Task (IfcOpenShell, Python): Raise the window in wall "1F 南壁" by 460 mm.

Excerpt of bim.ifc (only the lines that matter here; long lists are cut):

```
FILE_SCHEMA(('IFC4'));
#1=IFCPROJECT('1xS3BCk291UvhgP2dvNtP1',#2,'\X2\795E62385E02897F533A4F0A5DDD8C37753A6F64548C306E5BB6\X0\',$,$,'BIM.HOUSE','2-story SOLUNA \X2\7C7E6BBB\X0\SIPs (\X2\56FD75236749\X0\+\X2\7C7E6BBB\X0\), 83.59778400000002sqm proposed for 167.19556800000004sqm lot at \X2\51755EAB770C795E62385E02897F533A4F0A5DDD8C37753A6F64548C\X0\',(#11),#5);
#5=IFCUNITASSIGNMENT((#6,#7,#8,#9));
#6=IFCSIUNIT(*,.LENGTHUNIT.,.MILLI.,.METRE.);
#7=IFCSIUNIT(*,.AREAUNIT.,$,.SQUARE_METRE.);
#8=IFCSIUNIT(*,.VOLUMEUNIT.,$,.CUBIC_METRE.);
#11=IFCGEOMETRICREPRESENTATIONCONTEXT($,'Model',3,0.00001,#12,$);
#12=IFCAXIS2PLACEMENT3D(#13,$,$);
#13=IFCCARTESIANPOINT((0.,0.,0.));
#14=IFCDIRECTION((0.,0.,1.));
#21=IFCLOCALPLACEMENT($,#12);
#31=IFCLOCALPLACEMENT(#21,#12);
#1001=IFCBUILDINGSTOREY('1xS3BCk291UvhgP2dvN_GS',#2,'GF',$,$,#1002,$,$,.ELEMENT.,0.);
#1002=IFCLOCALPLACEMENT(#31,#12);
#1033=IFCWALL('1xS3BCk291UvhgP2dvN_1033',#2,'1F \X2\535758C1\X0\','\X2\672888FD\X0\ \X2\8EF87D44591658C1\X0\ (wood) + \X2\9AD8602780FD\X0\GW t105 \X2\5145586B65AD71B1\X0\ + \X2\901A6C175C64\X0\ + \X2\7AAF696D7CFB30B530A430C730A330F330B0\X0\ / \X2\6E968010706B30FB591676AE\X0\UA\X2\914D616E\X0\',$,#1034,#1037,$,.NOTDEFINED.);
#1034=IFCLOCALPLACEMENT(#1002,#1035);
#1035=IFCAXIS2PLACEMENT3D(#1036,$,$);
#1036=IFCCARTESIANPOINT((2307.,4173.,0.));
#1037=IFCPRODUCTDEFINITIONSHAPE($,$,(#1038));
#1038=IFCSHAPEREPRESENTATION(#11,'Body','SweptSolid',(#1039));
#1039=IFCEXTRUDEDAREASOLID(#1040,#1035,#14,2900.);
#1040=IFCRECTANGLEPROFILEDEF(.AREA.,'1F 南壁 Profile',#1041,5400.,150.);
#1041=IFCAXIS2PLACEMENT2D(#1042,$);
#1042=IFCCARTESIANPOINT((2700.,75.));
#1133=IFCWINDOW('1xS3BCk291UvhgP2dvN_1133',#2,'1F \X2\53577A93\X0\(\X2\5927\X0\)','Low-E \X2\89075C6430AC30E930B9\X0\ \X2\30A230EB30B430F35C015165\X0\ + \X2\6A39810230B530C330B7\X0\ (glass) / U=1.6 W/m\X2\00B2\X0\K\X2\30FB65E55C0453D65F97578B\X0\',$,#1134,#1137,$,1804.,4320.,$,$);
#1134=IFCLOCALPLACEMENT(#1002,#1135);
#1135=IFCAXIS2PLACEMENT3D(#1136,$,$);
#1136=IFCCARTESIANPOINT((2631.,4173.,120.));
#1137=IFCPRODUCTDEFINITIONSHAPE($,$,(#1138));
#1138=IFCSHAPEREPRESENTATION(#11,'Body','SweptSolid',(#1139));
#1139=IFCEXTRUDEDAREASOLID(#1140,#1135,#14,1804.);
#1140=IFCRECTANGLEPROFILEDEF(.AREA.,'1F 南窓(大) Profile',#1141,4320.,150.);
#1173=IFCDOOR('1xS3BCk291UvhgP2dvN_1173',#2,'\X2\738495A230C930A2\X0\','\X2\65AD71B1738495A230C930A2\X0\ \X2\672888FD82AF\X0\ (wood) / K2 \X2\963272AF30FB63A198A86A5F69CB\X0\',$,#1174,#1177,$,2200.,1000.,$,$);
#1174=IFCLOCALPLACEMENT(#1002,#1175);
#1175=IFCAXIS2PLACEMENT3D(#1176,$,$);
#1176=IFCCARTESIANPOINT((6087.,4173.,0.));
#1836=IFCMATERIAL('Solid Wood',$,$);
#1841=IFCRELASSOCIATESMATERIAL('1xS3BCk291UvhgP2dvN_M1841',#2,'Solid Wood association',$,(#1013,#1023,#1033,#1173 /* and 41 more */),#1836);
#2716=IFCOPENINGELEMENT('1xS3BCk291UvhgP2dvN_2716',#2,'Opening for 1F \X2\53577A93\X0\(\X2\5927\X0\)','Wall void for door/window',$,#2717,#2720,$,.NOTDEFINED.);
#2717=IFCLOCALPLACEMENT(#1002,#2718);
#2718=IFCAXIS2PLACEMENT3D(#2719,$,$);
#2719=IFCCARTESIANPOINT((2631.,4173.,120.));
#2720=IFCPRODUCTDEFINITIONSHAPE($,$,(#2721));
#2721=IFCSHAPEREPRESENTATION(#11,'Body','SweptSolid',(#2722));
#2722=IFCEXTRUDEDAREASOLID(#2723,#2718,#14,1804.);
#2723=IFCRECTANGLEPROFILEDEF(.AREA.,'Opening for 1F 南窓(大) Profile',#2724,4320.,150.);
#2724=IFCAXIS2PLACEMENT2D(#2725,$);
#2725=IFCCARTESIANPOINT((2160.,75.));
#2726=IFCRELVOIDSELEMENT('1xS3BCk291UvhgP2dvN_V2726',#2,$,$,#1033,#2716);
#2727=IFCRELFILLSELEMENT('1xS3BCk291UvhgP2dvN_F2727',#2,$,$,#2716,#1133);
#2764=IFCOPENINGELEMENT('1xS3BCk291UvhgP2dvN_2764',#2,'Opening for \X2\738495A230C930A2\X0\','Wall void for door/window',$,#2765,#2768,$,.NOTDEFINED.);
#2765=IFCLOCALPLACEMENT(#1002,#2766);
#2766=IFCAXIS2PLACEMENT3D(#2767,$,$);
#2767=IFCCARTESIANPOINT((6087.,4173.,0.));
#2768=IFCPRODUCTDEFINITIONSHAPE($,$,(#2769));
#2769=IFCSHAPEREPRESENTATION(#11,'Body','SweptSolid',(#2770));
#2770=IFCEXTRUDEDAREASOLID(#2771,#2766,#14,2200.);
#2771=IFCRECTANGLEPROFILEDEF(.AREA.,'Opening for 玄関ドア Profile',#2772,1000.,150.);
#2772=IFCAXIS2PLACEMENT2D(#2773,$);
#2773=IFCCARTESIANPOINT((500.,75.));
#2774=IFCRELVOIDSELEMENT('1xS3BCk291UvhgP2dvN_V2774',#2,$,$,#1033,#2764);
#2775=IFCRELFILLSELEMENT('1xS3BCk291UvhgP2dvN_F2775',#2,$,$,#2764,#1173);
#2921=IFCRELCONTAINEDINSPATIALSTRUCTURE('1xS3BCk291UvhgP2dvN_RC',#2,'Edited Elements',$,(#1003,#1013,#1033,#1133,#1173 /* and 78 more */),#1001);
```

```python
import numpy as np
import ifcopenshell
import ifcopenshell.api.geometry
import ifcopenshell.util.placement
import ifcopenshell.util.unit

model = ifcopenshell.open("bim.ifc")
unit_scale = ifcopenshell.util.unit.calculate_unit_scale(model)

window = model.by_guid("1xS3BCk291UvhgP2dvN_1133")
opening = window.FillsVoids[0].RelatingOpeningElement
dz = 460.0

shift = np.array([0.0, 0.0, dz])
# The window is not placed relative to its opening, so move both.
for product in (opening, window):
    matrix = ifcopenshell.util.placement.get_local_placement(product.ObjectPlacement)
    matrix[:3, 3] += shift
    ifcopenshell.api.geometry.edit_object_placement(model, product=product, matrix=matrix, is_si=False)

print(f"moved by {dz * unit_scale:+.3f} m")

model.write("bim_updated.ifc")
```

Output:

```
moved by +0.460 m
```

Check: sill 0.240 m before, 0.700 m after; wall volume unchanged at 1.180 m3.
